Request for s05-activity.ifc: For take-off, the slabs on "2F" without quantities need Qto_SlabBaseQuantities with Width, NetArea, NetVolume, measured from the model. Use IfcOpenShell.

First a look at what the model holds.

```python
import ifcopenshell
import ifcopenshell.util.element
import ifcopenshell.util.unit

model = ifcopenshell.open("s05-activity.ifc")
print(model.schema)
for unit_type in ("LENGTHUNIT", "AREAUNIT", "VOLUMEUNIT"):
    print(unit_type, ifcopenshell.util.unit.calculate_unit_scale(model, unit_type))
storey = next(s for s in model.by_type("IfcBuildingStorey") if s.Name == "2F")
slabs = [e for e in ifcopenshell.util.element.get_decomposition(storey) if e.is_a("IfcSlab")]
for e in sorted(slabs, key=lambda e: e.id()):
    print(e.id(), e.is_a(), e.Name, list(ifcopenshell.util.element.get_psets(e, qtos_only=True)), sep=" | ")
```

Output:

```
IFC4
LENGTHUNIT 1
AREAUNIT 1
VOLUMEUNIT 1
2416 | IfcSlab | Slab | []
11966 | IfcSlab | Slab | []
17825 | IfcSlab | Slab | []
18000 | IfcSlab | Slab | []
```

```python
import ifcopenshell
import ifcopenshell.api.pset
import ifcopenshell.geom
import ifcopenshell.util.element
import ifcopenshell.util.shape
import ifcopenshell.util.unit

model = ifcopenshell.open("s05-activity.ifc")
unit_scale = ifcopenshell.util.unit.calculate_unit_scale(model)
area_scale = ifcopenshell.util.unit.calculate_unit_scale(model, "AREAUNIT")
volume_scale = ifcopenshell.util.unit.calculate_unit_scale(model, "VOLUMEUNIT")
settings = ifcopenshell.geom.settings()

storey = next(s for s in model.by_type("IfcBuildingStorey") if s.Name == "2F")
slabs = [e for e in ifcopenshell.util.element.get_decomposition(storey) if e.is_a("IfcSlab")]

for e in sorted(slabs, key=lambda e: e.id()):
    if ifcopenshell.util.element.get_psets(e, qtos_only=True, should_inherit=False):
        continue
    # Geometry comes back in metres, in the element's own axes.
    shape = ifcopenshell.geom.create_shape(settings, e)
    values = {
        "Width": ifcopenshell.util.shape.get_z(shape.geometry) / unit_scale,
        "NetArea": ifcopenshell.util.shape.get_footprint_area(shape.geometry) / area_scale,
        "NetVolume": ifcopenshell.util.shape.get_volume(shape.geometry) / volume_scale,
    }
    qto = ifcopenshell.api.pset.add_qto(model, product=e, name="Qto_SlabBaseQuantities")
    ifcopenshell.api.pset.edit_qto(model, qto=qto, properties=values)
    print(e.id(), {k: round(v, 3) for k, v in values.items()})

model.write("s05-activity_edited.ifc")
```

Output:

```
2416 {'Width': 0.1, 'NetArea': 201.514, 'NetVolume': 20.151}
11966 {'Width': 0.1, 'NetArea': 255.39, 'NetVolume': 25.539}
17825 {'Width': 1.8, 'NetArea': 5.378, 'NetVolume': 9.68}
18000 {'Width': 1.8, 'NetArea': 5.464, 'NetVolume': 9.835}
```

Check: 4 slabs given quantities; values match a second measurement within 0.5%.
